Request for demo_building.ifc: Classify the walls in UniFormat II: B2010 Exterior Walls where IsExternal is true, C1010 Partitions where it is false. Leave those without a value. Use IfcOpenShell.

First a look at what the model holds.

```python
import ifcopenshell
import ifcopenshell.util.element

model = ifcopenshell.open("demo_building.ifc")
print(model.schema)
print("classifications:", [c.Name for c in model.by_type("IfcClassification")])
values = [ifcopenshell.util.element.get_pset(e, "Pset_WallCommon", "IsExternal") for e in model.by_type("IfcWall")]
for value in (True, False, None):
    print("IsExternal", value, values.count(value))
```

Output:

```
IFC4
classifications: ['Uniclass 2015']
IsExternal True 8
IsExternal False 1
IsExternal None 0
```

```python
import ifcopenshell
import ifcopenshell.api.classification
import ifcopenshell.util.element

model = ifcopenshell.open("demo_building.ifc")

system = ifcopenshell.api.classification.add_classification(model, classification="UniFormat II")

walls = model.by_type("IfcWall")
external = {e: ifcopenshell.util.element.get_pset(e, "Pset_WallCommon", "IsExternal") for e in walls}
for flag, code, name in ((True, "B2010", "Exterior Walls"), (False, "C1010", "Partitions")):
    products = [e for e in walls if external[e] is flag]
    ifcopenshell.api.classification.add_reference(
        model, products=products, classification=system, identification=code, name=name
    )
    print(code, len(products))

model.write("demo_building_v2.ifc")
```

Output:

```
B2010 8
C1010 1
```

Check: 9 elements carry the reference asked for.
